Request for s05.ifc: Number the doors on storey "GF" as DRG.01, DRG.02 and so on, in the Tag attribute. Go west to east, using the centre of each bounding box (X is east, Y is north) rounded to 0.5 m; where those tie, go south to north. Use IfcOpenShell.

First a look at what the model holds.

```python
import ifcopenshell
import ifcopenshell.util.element
import ifcopenshell.util.placement

model = ifcopenshell.open("s05.ifc")
print(model.schema)
storey = next(s for s in model.by_type("IfcBuildingStorey") if s.Name == "GF")
doors = [e for e in ifcopenshell.util.element.get_decomposition(storey) if e.is_a("IfcDoor")]
for e in sorted(doors, key=lambda e: e.id()):
    origin = ifcopenshell.util.placement.get_local_placement(e.ObjectPlacement)[:3, 3]
    print(e.id(), e.Tag, e.Name, origin.round(2) + 0.0, sep=" | ")
```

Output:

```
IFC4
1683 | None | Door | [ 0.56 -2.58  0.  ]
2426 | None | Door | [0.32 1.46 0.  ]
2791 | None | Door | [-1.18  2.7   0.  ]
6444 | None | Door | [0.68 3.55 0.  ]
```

```python
import ifcopenshell
import ifcopenshell.geom
import ifcopenshell.util.element
import ifcopenshell.util.shape

model = ifcopenshell.open("s05.ifc")
settings = ifcopenshell.geom.settings()
settings.set("use-world-coords", True)


def centre(element):
    shape = ifcopenshell.geom.create_shape(settings, element)
    return ifcopenshell.util.shape.get_bbox_centroid(shape.geometry)


storey = next(s for s in model.by_type("IfcBuildingStorey") if s.Name == "GF")
doors = [e for e in ifcopenshell.util.element.get_decomposition(storey) if e.is_a("IfcDoor")]

# Insertion points can sit at a corner or the storey origin, so sort by the geometry (in metres).
centres = {e: centre(e) for e in doors}
doors.sort(key=lambda e: (round(centres[e][0] / 0.5), centres[e][1]))

for i, e in enumerate(doors, start=1):
    number = f"DRG.{i:02d}"
    e.Tag = number
    print(e.id(), number)

model.write("s05_v2.ifc")
```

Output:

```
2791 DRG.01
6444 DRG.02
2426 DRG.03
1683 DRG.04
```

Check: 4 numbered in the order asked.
